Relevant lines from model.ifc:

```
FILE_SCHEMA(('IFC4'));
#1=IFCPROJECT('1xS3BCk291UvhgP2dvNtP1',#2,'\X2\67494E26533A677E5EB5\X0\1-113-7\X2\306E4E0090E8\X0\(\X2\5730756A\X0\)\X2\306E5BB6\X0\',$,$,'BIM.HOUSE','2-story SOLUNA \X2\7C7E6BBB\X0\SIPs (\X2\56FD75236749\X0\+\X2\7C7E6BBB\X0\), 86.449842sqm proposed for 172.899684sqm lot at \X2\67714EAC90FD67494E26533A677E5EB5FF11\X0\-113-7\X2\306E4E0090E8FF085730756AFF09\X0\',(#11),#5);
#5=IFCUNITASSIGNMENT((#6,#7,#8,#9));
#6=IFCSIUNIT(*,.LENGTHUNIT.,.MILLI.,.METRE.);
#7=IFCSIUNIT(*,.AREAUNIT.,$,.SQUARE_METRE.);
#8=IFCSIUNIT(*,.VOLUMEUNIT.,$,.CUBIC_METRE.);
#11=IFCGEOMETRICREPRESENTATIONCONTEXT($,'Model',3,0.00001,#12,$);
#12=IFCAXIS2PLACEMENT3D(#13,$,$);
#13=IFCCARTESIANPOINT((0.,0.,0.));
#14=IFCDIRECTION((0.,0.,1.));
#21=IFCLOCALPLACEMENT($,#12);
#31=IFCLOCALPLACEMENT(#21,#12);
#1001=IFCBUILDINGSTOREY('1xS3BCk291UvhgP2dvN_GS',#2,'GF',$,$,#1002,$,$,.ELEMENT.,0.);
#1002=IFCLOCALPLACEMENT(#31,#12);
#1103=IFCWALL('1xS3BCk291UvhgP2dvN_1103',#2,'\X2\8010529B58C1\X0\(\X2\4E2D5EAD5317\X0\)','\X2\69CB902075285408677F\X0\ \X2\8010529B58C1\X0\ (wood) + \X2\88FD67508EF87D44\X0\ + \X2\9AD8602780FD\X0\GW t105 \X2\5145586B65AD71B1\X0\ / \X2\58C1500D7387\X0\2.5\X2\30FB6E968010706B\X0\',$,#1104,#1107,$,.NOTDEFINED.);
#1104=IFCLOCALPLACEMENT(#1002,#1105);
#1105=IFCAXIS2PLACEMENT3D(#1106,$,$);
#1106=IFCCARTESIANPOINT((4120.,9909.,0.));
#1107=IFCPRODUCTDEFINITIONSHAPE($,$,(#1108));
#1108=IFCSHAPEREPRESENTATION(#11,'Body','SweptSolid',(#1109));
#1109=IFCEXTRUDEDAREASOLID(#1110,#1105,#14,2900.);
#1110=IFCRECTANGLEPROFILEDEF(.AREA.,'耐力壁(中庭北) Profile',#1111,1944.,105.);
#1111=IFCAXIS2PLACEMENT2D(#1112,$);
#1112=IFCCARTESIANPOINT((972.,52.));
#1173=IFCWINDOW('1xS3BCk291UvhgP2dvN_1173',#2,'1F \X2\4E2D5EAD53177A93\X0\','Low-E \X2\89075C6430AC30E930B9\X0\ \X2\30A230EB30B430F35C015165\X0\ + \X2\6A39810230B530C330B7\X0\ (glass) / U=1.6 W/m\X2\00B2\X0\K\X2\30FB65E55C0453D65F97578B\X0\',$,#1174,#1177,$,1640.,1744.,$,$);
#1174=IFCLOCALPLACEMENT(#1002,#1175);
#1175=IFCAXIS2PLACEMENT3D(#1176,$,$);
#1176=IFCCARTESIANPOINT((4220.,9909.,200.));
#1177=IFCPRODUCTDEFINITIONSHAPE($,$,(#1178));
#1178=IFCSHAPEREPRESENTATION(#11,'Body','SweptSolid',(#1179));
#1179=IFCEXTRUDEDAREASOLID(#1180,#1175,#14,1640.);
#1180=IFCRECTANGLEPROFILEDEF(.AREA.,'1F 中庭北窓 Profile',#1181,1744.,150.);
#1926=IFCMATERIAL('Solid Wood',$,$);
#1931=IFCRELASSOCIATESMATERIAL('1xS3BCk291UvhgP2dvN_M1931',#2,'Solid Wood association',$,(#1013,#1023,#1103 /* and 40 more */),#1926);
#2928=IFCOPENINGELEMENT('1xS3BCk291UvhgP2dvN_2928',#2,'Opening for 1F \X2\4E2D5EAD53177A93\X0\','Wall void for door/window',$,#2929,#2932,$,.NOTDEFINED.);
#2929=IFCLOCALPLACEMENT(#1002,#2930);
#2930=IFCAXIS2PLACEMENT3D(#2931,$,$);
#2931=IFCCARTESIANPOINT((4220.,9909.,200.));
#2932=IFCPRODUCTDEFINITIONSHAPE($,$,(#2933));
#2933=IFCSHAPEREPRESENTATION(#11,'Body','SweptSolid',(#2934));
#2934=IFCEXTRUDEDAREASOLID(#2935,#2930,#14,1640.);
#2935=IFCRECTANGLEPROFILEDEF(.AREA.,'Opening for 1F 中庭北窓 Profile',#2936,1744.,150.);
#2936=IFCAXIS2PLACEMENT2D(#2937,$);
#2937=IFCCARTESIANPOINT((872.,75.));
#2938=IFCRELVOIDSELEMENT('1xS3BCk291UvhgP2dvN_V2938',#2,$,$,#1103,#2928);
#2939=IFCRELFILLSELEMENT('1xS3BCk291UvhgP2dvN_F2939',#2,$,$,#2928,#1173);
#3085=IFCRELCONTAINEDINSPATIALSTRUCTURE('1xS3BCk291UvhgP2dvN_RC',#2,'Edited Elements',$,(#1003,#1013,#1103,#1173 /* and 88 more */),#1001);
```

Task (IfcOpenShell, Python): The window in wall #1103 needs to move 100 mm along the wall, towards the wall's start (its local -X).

```python
import ifcopenshell
import ifcopenshell.api.geometry
import ifcopenshell.util.placement

model = ifcopenshell.open("model.ifc")

window = model.by_guid("1xS3BCk291UvhgP2dvN_1173")
opening = window.FillsVoids[0].RelatingOpeningElement
wall = opening.VoidsElements[0].RelatingBuildingElement

wall_matrix = ifcopenshell.util.placement.get_local_placement(wall.ObjectPlacement)
shift = wall_matrix[:3, 0] * -100.0
before = ifcopenshell.util.placement.get_local_placement(window.ObjectPlacement)[:3, 3].copy()

# The window is not placed relative to its opening, so move both.
for product in (opening, window):
    matrix = ifcopenshell.util.placement.get_local_placement(product.ObjectPlacement)
    matrix[:3, 3] += shift
    ifcopenshell.api.geometry.edit_object_placement(model, product=product, matrix=matrix, is_si=False)

after = ifcopenshell.util.placement.get_local_placement(window.ObjectPlacement)[:3, 3]
print("window moved by", (after - before).round(3) + 0.0)

model.write("model_updated.ifc")
```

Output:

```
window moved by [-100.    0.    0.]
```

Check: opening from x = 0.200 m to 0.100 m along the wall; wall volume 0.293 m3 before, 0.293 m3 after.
